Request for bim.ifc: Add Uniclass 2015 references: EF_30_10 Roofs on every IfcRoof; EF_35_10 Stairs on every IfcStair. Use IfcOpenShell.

First a look at what the model holds.

```python
import ifcopenshell

model = ifcopenshell.open("bim.ifc")
print(model.schema)
print("classifications:", [c.Name for c in model.by_type("IfcClassification")])
for ifc_class in ("IfcDoor", "IfcRoof", "IfcStair", "IfcWall", "IfcWindow"):
    print(ifc_class, len(model.by_type(ifc_class)))
```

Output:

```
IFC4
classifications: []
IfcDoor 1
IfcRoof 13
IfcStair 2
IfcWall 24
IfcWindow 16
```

```python
import ifcopenshell
import ifcopenshell.api.classification

model = ifcopenshell.open("bim.ifc")

system = ifcopenshell.api.classification.add_classification(model, classification="Uniclass 2015")

codes = {
    "IfcRoof": ("EF_30_10", "Roofs"),
    "IfcStair": ("EF_35_10", "Stairs"),
}
for ifc_class, (code, name) in codes.items():
    products = model.by_type(ifc_class)
    ifcopenshell.api.classification.add_reference(
        model, products=products, classification=system, identification=code, name=name
    )
    print(code, len(products))

model.write("bim_rev.ifc")
```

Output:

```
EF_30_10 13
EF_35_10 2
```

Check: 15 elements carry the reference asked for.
